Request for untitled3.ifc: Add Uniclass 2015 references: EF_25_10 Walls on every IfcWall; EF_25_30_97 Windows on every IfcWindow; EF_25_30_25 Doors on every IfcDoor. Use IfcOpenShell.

First a look at what the model holds.

```python
import ifcopenshell

model = ifcopenshell.open("untitled3.ifc")
print(model.schema)
print("classifications:", [c.Name for c in model.by_type("IfcClassification")])
for ifc_class in ("IfcDoor", "IfcRoof", "IfcStair", "IfcWall", "IfcWindow"):
    print(ifc_class, len(model.by_type(ifc_class)))
```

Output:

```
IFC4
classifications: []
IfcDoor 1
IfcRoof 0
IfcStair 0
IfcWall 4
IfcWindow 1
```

```python
import ifcopenshell
import ifcopenshell.api.classification

model = ifcopenshell.open("untitled3.ifc")

system = ifcopenshell.api.classification.add_classification(model, classification="Uniclass 2015")

codes = {
    "IfcWall": ("EF_25_10", "Walls"),
    "IfcWindow": ("EF_25_30_97", "Windows"),
    "IfcDoor": ("EF_25_30_25", "Doors"),
}
for ifc_class, (code, name) in codes.items():
    products = model.by_type(ifc_class)
    ifcopenshell.api.classification.add_reference(
        model, products=products, classification=system, identification=code, name=name
    )
    print(code, len(products))

model.write("untitled3_rev.ifc")
```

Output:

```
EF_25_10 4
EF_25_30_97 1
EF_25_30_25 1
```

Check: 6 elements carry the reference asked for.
